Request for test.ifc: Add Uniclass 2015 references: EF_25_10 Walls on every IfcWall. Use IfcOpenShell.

First a look at what the model holds.

```python
import ifcopenshell

model = ifcopenshell.open("test.ifc")
print(model.schema)
print("classifications:", [c.Name for c in model.by_type("IfcClassification")])
for ifc_class in ("IfcDoor", "IfcRoof", "IfcStair", "IfcWall", "IfcWindow"):
    print(ifc_class, len(model.by_type(ifc_class)))
```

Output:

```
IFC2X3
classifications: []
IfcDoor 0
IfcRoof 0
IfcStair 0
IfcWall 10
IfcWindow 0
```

```python
import ifcopenshell
import ifcopenshell.api.classification

model = ifcopenshell.open("test.ifc")

# IFC2X3 requires Source and Edition and has no link from the project to the system.
system = model.create_entity("IfcClassification", Source="NBS", Edition="2015", Name="Uniclass 2015")

codes = {
    "IfcWall": ("EF_25_10", "Walls"),
}
for ifc_class, (code, name) in codes.items():
    products = model.by_type(ifc_class)
    ifcopenshell.api.classification.add_reference(
        model, products=products, classification=system, identification=code, name=name
    )
    print(code, len(products))

model.write("test-out.ifc")
```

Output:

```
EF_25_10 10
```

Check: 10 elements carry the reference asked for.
